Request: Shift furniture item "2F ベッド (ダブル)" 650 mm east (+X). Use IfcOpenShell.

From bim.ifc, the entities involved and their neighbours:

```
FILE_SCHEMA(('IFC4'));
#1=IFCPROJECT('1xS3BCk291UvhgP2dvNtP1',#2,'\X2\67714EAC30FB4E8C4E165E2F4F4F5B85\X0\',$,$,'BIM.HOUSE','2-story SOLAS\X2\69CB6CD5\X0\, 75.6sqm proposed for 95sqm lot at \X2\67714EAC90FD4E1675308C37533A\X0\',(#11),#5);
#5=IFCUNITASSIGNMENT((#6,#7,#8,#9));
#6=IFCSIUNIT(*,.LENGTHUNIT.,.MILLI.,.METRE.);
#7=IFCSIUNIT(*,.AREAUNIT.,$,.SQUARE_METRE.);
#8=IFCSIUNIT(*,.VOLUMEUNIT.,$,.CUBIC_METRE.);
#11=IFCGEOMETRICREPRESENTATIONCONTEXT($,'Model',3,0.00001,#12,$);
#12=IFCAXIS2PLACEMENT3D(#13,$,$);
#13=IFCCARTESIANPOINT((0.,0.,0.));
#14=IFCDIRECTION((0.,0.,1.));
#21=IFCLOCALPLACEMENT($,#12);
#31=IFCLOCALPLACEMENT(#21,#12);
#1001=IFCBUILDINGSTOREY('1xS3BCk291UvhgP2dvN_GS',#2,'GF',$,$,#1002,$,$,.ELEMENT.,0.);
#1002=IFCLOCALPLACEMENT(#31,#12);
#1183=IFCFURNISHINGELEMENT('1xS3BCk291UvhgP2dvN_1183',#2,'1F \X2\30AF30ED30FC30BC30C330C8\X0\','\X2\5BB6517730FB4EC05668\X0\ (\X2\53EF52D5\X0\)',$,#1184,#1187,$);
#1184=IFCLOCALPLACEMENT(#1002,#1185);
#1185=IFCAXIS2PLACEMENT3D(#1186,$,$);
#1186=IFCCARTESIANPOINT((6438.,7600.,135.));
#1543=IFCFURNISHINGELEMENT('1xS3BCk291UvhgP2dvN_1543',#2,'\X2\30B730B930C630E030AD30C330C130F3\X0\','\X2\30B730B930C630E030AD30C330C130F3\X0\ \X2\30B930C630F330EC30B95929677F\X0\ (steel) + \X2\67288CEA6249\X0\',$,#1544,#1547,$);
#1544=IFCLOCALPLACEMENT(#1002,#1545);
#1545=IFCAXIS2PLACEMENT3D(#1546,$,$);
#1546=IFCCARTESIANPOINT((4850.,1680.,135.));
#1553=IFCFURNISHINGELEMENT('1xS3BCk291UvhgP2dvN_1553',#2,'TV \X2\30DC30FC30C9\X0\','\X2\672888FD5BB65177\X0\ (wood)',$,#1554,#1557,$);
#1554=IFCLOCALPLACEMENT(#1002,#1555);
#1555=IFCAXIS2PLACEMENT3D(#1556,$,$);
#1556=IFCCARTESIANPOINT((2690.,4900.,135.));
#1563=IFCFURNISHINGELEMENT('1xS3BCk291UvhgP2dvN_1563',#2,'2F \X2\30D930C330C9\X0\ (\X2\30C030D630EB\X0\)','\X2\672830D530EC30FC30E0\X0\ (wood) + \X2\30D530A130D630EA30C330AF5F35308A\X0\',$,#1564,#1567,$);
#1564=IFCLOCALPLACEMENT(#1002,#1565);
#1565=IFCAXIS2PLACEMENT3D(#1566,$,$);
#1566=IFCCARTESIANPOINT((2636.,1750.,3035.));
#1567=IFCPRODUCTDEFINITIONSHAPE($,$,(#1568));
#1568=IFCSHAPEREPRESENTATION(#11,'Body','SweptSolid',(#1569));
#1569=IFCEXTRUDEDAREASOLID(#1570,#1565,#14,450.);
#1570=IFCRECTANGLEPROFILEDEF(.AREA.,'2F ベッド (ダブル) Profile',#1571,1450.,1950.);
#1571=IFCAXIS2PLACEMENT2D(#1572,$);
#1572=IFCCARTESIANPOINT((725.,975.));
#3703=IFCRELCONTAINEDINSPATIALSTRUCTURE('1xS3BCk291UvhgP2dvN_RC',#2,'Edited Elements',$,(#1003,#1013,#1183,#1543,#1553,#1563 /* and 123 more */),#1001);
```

```python
import ifcopenshell
import ifcopenshell.api.geometry
import ifcopenshell.util.placement

model = ifcopenshell.open("bim.ifc")

item = model.by_id(1563)
matrix = ifcopenshell.util.placement.get_local_placement(item.ObjectPlacement)
matrix[0, 3] += 650.0
ifcopenshell.api.geometry.edit_object_placement(model, product=item, matrix=matrix, is_si=False)

print(ifcopenshell.util.placement.get_local_placement(item.ObjectPlacement).round(3) + 0.0)

model.write("bim_rev.ifc")
```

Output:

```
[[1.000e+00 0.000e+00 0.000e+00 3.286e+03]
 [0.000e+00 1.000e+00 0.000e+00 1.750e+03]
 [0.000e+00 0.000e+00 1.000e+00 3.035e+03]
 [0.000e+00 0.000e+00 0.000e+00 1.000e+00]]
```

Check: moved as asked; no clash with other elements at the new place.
